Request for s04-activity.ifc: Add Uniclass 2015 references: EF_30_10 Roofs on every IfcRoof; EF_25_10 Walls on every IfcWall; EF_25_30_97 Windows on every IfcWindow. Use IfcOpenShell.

First a look at what the model holds.

```python
import ifcopenshell

model = ifcopenshell.open("s04-activity.ifc")
print(model.schema)
print("classifications:", [c.Name for c in model.by_type("IfcClassification")])
for ifc_class in ("IfcDoor", "IfcRoof", "IfcStair", "IfcWall", "IfcWindow"):
    print(ifc_class, len(model.by_type(ifc_class)))
```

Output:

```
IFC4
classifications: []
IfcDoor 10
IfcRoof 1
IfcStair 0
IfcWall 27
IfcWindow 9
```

```python
import ifcopenshell
import ifcopenshell.api.classification

model = ifcopenshell.open("s04-activity.ifc")

system = ifcopenshell.api.classification.add_classification(model, classification="Uniclass 2015")

codes = {
    "IfcRoof": ("EF_30_10", "Roofs"),
    "IfcWall": ("EF_25_10", "Walls"),
    "IfcWindow": ("EF_25_30_97", "Windows"),
}
for ifc_class, (code, name) in codes.items():
    products = model.by_type(ifc_class)
    ifcopenshell.api.classification.add_reference(
        model, products=products, classification=system, identification=code, name=name
    )
    print(code, len(products))

model.write("s04-activity_rev.ifc")
```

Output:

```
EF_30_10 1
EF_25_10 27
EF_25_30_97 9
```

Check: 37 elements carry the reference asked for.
